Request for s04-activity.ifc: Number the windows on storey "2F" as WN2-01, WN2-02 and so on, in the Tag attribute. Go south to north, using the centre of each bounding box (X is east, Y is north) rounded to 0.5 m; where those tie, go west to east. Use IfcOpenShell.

First a look at what the model holds.

```python
import ifcopenshell
import ifcopenshell.util.element
import ifcopenshell.util.placement

model = ifcopenshell.open("s04-activity.ifc")
print(model.schema)
storey = next(s for s in model.by_type("IfcBuildingStorey") if s.Name == "2F")
windows = [e for e in ifcopenshell.util.element.get_decomposition(storey) if e.is_a("IfcWindow")]
for e in sorted(windows, key=lambda e: e.id()):
    origin = ifcopenshell.util.placement.get_local_placement(e.ObjectPlacement)[:3, 3]
    print(e.id(), e.Tag, e.Name, origin.round(2) + 0.0, sep=" | ")
```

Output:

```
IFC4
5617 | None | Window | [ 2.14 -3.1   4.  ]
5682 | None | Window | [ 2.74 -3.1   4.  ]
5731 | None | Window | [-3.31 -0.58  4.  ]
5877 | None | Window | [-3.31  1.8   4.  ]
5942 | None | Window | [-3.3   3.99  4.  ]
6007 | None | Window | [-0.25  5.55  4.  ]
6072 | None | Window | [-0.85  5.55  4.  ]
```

```python
import ifcopenshell
import ifcopenshell.geom
import ifcopenshell.util.element
import ifcopenshell.util.shape

model = ifcopenshell.open("s04-activity.ifc")
settings = ifcopenshell.geom.settings()
settings.set("use-world-coords", True)


def centre(element):
    shape = ifcopenshell.geom.create_shape(settings, element)
    return ifcopenshell.util.shape.get_bbox_centroid(shape.geometry)


storey = next(s for s in model.by_type("IfcBuildingStorey") if s.Name == "2F")
windows = [e for e in ifcopenshell.util.element.get_decomposition(storey) if e.is_a("IfcWindow")]

# Insertion points can sit at a corner or the storey origin, so sort by the geometry (in metres).
centres = {e: centre(e) for e in windows}
windows.sort(key=lambda e: (round(centres[e][1] / 0.5), centres[e][0]))

for i, e in enumerate(windows, start=1):
    number = f"WN2-{i:02d}"
    e.Tag = number
    print(e.id(), number)

model.write("s04-activity_updated.ifc")
```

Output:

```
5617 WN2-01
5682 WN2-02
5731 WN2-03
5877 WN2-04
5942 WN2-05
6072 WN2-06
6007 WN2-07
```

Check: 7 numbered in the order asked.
